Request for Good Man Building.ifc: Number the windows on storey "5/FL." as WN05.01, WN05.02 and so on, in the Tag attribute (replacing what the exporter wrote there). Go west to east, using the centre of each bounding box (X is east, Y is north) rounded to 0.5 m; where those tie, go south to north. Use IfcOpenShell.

First a look at what the model holds.

```python
import ifcopenshell
import ifcopenshell.util.element
import ifcopenshell.util.placement

model = ifcopenshell.open("Good Man Building.ifc")
print(model.schema)
storey = next(s for s in model.by_type("IfcBuildingStorey") if s.Name == "5/FL.")
windows = [e for e in ifcopenshell.util.element.get_decomposition(storey) if e.is_a("IfcWindow")]
for e in sorted(windows, key=lambda e: e.id()):
    origin = ifcopenshell.util.placement.get_local_placement(e.ObjectPlacement)[:3, 3]
    print(e.id(), e.Tag, e.Name, origin.round(2) + 0.0, sep=" | ")
```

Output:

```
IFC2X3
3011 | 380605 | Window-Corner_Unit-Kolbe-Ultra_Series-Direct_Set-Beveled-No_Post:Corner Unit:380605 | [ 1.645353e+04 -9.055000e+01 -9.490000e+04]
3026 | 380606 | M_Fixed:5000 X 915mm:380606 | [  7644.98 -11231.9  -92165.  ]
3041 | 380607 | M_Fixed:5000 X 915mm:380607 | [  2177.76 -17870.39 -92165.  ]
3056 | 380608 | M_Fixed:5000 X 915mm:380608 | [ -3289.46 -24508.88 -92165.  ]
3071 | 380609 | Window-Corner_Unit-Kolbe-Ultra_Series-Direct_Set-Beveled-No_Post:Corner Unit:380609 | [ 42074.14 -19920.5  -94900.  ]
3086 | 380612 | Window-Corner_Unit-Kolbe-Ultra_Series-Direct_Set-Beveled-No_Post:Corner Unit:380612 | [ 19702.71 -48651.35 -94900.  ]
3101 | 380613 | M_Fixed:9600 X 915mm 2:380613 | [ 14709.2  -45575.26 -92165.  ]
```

```python
import ifcopenshell
import ifcopenshell.geom
import ifcopenshell.util.element
import ifcopenshell.util.shape

model = ifcopenshell.open("Good Man Building.ifc")
settings = ifcopenshell.geom.settings()
settings.set("use-world-coords", True)


def centre(element):
    shape = ifcopenshell.geom.create_shape(settings, element)
    return ifcopenshell.util.shape.get_bbox_centroid(shape.geometry)


storey = next(s for s in model.by_type("IfcBuildingStorey") if s.Name == "5/FL.")
windows = [e for e in ifcopenshell.util.element.get_decomposition(storey) if e.is_a("IfcWindow")]

# Insertion points can sit at a corner or the storey origin, so sort by the geometry (in metres).
centres = {e: centre(e) for e in windows}
windows.sort(key=lambda e: (round(centres[e][0] / 0.5), centres[e][1]))

for i, e in enumerate(windows, start=1):
    number = f"WN05.{i:02d}"
    e.Tag = number
    print(e.id(), number)

model.write("Good Man Building_edited.ifc")
```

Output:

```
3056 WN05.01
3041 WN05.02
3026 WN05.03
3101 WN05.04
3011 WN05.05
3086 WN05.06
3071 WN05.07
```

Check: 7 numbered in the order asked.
